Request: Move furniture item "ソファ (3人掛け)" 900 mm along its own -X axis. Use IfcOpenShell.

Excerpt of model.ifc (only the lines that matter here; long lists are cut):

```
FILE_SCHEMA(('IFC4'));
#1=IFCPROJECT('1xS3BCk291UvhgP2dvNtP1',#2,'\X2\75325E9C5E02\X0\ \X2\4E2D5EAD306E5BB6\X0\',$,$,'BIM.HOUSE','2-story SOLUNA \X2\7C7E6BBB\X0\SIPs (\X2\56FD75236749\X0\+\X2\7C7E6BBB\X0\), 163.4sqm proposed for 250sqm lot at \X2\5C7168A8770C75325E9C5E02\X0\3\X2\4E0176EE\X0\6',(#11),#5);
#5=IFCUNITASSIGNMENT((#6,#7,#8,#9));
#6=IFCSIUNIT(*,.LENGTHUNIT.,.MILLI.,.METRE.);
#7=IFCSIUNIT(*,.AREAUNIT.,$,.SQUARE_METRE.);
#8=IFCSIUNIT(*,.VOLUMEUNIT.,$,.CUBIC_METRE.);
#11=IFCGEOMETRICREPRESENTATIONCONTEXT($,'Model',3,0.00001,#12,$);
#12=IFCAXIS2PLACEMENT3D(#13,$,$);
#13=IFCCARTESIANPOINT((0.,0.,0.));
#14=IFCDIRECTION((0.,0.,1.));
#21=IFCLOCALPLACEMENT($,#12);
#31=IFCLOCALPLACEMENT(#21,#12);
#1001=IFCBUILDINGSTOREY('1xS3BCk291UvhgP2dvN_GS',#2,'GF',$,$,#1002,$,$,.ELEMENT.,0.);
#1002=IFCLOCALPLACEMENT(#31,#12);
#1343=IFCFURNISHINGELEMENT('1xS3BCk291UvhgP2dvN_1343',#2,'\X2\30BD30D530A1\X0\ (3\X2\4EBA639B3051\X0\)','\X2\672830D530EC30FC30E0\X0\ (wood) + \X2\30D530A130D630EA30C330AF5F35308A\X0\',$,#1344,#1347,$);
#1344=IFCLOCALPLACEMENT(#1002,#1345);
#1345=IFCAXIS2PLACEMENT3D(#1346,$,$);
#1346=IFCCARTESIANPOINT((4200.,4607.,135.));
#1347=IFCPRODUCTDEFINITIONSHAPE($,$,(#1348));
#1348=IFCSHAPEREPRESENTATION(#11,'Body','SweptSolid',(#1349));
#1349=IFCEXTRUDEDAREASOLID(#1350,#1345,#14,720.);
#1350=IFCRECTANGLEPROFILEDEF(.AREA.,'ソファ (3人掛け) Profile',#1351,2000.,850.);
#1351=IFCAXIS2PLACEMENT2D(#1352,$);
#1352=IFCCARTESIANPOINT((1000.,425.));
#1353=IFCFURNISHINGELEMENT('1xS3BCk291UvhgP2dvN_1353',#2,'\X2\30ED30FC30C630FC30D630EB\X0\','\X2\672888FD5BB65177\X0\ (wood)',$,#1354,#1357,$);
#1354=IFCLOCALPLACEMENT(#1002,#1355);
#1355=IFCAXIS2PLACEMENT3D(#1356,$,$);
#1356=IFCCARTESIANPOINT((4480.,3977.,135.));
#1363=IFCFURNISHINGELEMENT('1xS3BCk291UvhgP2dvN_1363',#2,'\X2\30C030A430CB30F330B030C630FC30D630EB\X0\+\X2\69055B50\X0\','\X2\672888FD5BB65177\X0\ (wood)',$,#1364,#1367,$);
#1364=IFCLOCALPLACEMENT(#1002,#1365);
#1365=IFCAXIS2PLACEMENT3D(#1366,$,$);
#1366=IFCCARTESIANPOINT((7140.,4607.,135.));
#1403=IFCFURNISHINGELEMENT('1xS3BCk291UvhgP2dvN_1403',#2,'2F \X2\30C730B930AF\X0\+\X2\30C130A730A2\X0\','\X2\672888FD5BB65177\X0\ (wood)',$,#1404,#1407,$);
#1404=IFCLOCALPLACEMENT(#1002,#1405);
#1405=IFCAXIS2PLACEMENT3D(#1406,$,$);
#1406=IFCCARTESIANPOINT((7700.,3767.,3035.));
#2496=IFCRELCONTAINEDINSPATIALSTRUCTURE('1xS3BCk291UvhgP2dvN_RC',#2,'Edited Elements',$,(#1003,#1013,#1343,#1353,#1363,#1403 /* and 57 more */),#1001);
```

```python
import ifcopenshell
import ifcopenshell.api.geometry
import ifcopenshell.util.placement
import ifcopenshell.util.unit

model = ifcopenshell.open("model.ifc")
unit_scale = ifcopenshell.util.unit.calculate_unit_scale(model)

item = model.by_guid("1xS3BCk291UvhgP2dvN_1343")
matrix = ifcopenshell.util.placement.get_local_placement(item.ObjectPlacement)
matrix[:3, 3] -= matrix[:3, 0] * 0.9 / unit_scale
ifcopenshell.api.geometry.edit_object_placement(model, product=item, matrix=matrix, is_si=False)

print(ifcopenshell.util.placement.get_local_placement(item.ObjectPlacement).round(3) + 0.0)

model.write("model_updated.ifc")
```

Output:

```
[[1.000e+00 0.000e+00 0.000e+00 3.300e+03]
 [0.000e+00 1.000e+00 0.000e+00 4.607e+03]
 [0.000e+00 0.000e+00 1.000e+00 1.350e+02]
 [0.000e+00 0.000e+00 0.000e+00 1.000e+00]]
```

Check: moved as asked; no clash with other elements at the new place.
